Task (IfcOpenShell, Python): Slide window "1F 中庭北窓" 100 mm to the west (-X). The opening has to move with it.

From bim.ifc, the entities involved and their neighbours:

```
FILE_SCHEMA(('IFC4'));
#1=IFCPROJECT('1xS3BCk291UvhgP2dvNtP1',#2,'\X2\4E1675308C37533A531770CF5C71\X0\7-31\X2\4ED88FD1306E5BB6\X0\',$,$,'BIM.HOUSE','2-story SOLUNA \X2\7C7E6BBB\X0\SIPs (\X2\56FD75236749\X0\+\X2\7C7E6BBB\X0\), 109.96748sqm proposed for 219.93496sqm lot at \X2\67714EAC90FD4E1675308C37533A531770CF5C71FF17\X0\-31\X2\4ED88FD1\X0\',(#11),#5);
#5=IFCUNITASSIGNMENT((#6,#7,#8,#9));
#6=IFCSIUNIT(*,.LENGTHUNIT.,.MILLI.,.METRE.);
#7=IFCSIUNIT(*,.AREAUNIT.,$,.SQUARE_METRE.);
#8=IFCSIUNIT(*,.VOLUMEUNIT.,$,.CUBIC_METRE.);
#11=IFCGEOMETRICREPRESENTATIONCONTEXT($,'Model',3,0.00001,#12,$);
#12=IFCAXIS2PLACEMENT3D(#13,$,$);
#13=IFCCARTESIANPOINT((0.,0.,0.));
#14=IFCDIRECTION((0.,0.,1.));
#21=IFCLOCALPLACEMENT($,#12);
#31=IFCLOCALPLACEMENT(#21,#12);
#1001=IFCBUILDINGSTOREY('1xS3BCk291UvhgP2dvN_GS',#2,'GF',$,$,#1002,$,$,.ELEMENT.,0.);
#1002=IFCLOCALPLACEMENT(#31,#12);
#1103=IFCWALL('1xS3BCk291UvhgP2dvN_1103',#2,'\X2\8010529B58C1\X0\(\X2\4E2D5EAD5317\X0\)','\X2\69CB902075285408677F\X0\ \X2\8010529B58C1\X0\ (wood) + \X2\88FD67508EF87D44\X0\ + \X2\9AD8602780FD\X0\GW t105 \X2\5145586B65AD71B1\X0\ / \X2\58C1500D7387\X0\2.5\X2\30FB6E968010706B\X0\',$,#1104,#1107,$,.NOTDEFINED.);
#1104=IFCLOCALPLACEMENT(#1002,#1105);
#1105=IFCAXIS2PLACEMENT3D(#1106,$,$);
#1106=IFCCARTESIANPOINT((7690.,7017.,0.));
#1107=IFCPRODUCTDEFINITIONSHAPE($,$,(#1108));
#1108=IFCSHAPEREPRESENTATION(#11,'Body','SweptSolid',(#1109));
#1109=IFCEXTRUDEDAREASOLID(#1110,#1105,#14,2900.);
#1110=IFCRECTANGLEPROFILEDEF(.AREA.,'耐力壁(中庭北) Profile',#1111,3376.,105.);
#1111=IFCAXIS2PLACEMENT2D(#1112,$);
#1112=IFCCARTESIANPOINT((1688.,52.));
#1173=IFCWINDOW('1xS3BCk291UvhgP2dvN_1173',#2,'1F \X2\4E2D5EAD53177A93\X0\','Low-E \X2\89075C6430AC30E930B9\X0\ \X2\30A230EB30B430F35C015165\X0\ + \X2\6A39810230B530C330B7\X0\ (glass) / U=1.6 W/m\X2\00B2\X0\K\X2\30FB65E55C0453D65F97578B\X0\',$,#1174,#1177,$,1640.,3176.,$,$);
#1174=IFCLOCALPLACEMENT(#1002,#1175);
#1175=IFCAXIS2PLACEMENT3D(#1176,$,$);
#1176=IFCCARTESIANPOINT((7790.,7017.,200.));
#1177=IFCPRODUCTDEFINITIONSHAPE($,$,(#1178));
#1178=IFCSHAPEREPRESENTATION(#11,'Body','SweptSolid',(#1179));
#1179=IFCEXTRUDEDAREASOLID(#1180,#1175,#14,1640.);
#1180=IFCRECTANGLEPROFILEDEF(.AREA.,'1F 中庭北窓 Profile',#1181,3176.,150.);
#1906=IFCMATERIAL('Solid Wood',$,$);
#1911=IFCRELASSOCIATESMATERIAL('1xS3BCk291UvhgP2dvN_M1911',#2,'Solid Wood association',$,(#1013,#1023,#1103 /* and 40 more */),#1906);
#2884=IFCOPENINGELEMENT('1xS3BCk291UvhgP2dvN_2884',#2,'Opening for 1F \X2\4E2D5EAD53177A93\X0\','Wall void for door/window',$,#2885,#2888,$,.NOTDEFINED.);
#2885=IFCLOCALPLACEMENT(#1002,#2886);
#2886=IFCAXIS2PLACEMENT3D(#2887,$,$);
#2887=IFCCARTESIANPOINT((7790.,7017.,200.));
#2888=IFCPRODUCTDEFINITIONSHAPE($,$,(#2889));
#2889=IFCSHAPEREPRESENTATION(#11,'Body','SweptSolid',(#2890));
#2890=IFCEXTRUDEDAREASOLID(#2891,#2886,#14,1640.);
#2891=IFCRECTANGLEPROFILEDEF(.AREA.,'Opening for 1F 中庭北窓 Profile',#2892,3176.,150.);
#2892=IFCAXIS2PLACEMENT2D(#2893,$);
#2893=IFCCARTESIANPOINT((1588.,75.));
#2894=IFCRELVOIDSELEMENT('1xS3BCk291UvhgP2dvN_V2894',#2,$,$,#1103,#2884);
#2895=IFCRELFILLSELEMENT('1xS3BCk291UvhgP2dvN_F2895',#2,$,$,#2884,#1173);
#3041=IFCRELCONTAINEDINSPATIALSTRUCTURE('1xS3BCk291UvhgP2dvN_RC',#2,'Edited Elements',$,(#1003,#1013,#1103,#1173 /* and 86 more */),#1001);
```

```python
import ifcopenshell
import ifcopenshell.api.geometry
import ifcopenshell.util.placement
import ifcopenshell.util.unit

model = ifcopenshell.open("bim.ifc")
unit_scale = ifcopenshell.util.unit.calculate_unit_scale(model)

window = model.by_guid("1xS3BCk291UvhgP2dvN_1173")
opening = window.FillsVoids[0].RelatingOpeningElement
wall = opening.VoidsElements[0].RelatingBuildingElement

wall_matrix = ifcopenshell.util.placement.get_local_placement(wall.ObjectPlacement)
shift = wall_matrix[:3, 0] * -0.1 / unit_scale
before = ifcopenshell.util.placement.get_local_placement(window.ObjectPlacement)[:3, 3].copy()

# The window is not placed relative to its opening, so move both.
for product in (opening, window):
    matrix = ifcopenshell.util.placement.get_local_placement(product.ObjectPlacement)
    matrix[:3, 3] += shift
    ifcopenshell.api.geometry.edit_object_placement(model, product=product, matrix=matrix, is_si=False)

after = ifcopenshell.util.placement.get_local_placement(window.ObjectPlacement)[:3, 3]
print("window moved by", (after - before).round(3) + 0.0)

model.write("bim_edited.ifc")
```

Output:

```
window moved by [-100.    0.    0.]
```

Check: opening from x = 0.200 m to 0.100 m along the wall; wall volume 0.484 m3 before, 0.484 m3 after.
